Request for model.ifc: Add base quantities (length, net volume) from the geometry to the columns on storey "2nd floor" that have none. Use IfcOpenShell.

First a look at what the model holds.

```python
import ifcopenshell
import ifcopenshell.util.element
import ifcopenshell.util.unit

model = ifcopenshell.open("model.ifc")
print(model.schema)
for unit_type in ("LENGTHUNIT", "AREAUNIT", "VOLUMEUNIT"):
    print(unit_type, ifcopenshell.util.unit.calculate_unit_scale(model, unit_type))
storey = next(s for s in model.by_type("IfcBuildingStorey") if s.Name == "2nd floor")
columns = [e for e in ifcopenshell.util.element.get_decomposition(storey) if e.is_a("IfcColumn")]
for e in sorted(columns, key=lambda e: e.id()):
    print(e.id(), e.is_a(), e.Name, list(ifcopenshell.util.element.get_psets(e, qtos_only=True)), sep=" | ")
```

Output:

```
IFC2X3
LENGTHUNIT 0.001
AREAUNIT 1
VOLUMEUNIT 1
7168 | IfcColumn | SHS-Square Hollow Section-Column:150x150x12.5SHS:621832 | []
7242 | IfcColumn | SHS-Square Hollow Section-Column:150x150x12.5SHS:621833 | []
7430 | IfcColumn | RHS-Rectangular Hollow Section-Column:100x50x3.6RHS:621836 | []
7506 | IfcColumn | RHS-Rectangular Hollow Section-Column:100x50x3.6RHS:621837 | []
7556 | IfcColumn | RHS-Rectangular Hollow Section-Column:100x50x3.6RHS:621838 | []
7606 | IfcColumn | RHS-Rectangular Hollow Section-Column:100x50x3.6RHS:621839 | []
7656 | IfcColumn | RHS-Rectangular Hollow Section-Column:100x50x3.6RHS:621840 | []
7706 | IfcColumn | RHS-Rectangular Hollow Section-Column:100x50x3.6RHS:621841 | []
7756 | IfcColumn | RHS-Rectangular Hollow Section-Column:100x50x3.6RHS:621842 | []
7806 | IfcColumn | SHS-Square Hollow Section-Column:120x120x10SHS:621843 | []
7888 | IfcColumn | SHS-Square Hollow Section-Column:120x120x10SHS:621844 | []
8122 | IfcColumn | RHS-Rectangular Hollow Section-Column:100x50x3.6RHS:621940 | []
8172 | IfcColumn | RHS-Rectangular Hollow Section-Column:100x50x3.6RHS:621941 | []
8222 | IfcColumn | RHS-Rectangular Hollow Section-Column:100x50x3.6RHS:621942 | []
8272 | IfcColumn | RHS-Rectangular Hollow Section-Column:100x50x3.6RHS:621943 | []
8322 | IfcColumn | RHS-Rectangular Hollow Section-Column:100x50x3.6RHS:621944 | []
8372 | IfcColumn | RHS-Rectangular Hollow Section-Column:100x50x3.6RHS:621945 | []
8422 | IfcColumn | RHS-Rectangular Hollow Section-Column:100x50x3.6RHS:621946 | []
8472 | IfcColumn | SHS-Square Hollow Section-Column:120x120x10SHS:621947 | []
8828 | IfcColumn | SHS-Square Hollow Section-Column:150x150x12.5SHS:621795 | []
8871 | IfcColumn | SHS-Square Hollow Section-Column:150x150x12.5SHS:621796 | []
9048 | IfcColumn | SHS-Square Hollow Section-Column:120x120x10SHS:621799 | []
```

```python
import ifcopenshell
import ifcopenshell.api.pset
import ifcopenshell.geom
import ifcopenshell.util.element
import ifcopenshell.util.shape
import ifcopenshell.util.unit

model = ifcopenshell.open("model.ifc")
unit_scale = ifcopenshell.util.unit.calculate_unit_scale(model)
volume_scale = ifcopenshell.util.unit.calculate_unit_scale(model, "VOLUMEUNIT")
settings = ifcopenshell.geom.settings()

storey = next(s for s in model.by_type("IfcBuildingStorey") if s.Name == "2nd floor")
columns = [e for e in ifcopenshell.util.element.get_decomposition(storey) if e.is_a("IfcColumn")]

for e in sorted(columns, key=lambda e: e.id()):
    if ifcopenshell.util.element.get_psets(e, qtos_only=True, should_inherit=False):
        continue
    # Geometry comes back in metres, in the element's own axes.
    shape = ifcopenshell.geom.create_shape(settings, e)
    values = {
        "Length": ifcopenshell.util.shape.get_z(shape.geometry) / unit_scale,
        "NetVolume": ifcopenshell.util.shape.get_volume(shape.geometry) / volume_scale,
    }
    qto = ifcopenshell.api.pset.add_qto(model, product=e, name="BaseQuantities")
    ifcopenshell.api.pset.edit_qto(model, qto=qto, properties=values)
    print(e.id(), {k: round(v, 3) for k, v in values.items()})

model.write("model_updated.ifc")
```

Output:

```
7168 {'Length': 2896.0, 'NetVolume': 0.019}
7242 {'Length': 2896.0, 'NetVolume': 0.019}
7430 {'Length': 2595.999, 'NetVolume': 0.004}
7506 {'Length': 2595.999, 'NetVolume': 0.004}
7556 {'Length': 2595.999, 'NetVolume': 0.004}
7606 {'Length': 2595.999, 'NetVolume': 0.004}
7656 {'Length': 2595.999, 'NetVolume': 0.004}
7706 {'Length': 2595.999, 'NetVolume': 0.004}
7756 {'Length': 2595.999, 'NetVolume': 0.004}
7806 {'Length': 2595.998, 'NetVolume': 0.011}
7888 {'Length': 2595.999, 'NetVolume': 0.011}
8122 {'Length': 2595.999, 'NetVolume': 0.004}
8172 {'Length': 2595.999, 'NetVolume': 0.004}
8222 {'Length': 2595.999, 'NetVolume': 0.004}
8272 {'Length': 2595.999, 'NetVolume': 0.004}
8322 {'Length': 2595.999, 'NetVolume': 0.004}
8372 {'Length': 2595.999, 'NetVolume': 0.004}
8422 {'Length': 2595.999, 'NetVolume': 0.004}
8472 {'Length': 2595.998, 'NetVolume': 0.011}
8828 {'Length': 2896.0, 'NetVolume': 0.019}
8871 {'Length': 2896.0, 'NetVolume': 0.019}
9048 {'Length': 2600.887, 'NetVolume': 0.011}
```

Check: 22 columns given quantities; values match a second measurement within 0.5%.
